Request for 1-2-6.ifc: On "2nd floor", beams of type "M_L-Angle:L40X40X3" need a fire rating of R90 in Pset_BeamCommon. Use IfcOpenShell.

First a look at what the model holds.

```python
import ifcopenshell
import ifcopenshell.util.element

model = ifcopenshell.open("1-2-6.ifc")
print(model.schema)
storey = next(s for s in model.by_type("IfcBuildingStorey") if s.Name == "2nd floor")
beams = [e for e in ifcopenshell.util.element.get_decomposition(storey) if e.is_a("IfcBeam")]
seen = {}
for e in beams:
    element_type = ifcopenshell.util.element.get_type(e)
    key = (element_type.Name if element_type != e and element_type else None, ifcopenshell.util.element.get_pset(e, "Pset_BeamCommon", "FireRating"))
    seen[key] = seen.get(key, 0) + 1
for (name, value), count in sorted(seen.items(), key=str):
    print(count, "x", name, "|", value)
```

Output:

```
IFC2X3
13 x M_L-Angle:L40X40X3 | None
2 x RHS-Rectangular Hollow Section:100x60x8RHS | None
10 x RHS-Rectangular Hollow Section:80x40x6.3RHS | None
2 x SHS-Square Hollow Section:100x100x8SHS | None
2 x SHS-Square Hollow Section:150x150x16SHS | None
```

```python
import ifcopenshell
import ifcopenshell.api.pset
import ifcopenshell.util.element

model = ifcopenshell.open("1-2-6.ifc")

storey = next(s for s in model.by_type("IfcBuildingStorey") if s.Name == "2nd floor")
beams = [e for e in ifcopenshell.util.element.get_decomposition(storey) if e.is_a("IfcBeam")]

count = 0
for e in beams:
    element_type = ifcopenshell.util.element.get_type(e)
    if element_type in (None, e) or element_type.Name != "M_L-Angle:L40X40X3":
        continue
    # add_pset returns the element's existing set when there is one.
    pset = ifcopenshell.api.pset.add_pset(model, product=e, name="Pset_BeamCommon")
    ifcopenshell.api.pset.edit_pset(model, pset=pset, properties={"FireRating": "R90"})
    count += 1

print(count, "beams updated")

model.write("1-2-6-out.ifc")
```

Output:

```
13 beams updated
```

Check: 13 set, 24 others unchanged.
